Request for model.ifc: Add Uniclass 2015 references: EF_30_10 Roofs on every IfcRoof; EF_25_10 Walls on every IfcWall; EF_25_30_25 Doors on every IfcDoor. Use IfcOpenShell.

First a look at what the model holds.

```python
import ifcopenshell

model = ifcopenshell.open("model.ifc")
print(model.schema)
print("classifications:", [c.Name for c in model.by_type("IfcClassification")])
for ifc_class in ("IfcDoor", "IfcRoof", "IfcStair", "IfcWall", "IfcWindow"):
    print(ifc_class, len(model.by_type(ifc_class)))
```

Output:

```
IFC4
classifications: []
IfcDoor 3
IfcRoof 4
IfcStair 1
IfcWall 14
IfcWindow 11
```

```python
import ifcopenshell
import ifcopenshell.api.classification

model = ifcopenshell.open("model.ifc")

system = ifcopenshell.api.classification.add_classification(model, classification="Uniclass 2015")

codes = {
    "IfcRoof": ("EF_30_10", "Roofs"),
    "IfcWall": ("EF_25_10", "Walls"),
    "IfcDoor": ("EF_25_30_25", "Doors"),
}
for ifc_class, (code, name) in codes.items():
    products = model.by_type(ifc_class)
    ifcopenshell.api.classification.add_reference(
        model, products=products, classification=system, identification=code, name=name
    )
    print(code, len(products))

model.write("model_updated.ifc")
```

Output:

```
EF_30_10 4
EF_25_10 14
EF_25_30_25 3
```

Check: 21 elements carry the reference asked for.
